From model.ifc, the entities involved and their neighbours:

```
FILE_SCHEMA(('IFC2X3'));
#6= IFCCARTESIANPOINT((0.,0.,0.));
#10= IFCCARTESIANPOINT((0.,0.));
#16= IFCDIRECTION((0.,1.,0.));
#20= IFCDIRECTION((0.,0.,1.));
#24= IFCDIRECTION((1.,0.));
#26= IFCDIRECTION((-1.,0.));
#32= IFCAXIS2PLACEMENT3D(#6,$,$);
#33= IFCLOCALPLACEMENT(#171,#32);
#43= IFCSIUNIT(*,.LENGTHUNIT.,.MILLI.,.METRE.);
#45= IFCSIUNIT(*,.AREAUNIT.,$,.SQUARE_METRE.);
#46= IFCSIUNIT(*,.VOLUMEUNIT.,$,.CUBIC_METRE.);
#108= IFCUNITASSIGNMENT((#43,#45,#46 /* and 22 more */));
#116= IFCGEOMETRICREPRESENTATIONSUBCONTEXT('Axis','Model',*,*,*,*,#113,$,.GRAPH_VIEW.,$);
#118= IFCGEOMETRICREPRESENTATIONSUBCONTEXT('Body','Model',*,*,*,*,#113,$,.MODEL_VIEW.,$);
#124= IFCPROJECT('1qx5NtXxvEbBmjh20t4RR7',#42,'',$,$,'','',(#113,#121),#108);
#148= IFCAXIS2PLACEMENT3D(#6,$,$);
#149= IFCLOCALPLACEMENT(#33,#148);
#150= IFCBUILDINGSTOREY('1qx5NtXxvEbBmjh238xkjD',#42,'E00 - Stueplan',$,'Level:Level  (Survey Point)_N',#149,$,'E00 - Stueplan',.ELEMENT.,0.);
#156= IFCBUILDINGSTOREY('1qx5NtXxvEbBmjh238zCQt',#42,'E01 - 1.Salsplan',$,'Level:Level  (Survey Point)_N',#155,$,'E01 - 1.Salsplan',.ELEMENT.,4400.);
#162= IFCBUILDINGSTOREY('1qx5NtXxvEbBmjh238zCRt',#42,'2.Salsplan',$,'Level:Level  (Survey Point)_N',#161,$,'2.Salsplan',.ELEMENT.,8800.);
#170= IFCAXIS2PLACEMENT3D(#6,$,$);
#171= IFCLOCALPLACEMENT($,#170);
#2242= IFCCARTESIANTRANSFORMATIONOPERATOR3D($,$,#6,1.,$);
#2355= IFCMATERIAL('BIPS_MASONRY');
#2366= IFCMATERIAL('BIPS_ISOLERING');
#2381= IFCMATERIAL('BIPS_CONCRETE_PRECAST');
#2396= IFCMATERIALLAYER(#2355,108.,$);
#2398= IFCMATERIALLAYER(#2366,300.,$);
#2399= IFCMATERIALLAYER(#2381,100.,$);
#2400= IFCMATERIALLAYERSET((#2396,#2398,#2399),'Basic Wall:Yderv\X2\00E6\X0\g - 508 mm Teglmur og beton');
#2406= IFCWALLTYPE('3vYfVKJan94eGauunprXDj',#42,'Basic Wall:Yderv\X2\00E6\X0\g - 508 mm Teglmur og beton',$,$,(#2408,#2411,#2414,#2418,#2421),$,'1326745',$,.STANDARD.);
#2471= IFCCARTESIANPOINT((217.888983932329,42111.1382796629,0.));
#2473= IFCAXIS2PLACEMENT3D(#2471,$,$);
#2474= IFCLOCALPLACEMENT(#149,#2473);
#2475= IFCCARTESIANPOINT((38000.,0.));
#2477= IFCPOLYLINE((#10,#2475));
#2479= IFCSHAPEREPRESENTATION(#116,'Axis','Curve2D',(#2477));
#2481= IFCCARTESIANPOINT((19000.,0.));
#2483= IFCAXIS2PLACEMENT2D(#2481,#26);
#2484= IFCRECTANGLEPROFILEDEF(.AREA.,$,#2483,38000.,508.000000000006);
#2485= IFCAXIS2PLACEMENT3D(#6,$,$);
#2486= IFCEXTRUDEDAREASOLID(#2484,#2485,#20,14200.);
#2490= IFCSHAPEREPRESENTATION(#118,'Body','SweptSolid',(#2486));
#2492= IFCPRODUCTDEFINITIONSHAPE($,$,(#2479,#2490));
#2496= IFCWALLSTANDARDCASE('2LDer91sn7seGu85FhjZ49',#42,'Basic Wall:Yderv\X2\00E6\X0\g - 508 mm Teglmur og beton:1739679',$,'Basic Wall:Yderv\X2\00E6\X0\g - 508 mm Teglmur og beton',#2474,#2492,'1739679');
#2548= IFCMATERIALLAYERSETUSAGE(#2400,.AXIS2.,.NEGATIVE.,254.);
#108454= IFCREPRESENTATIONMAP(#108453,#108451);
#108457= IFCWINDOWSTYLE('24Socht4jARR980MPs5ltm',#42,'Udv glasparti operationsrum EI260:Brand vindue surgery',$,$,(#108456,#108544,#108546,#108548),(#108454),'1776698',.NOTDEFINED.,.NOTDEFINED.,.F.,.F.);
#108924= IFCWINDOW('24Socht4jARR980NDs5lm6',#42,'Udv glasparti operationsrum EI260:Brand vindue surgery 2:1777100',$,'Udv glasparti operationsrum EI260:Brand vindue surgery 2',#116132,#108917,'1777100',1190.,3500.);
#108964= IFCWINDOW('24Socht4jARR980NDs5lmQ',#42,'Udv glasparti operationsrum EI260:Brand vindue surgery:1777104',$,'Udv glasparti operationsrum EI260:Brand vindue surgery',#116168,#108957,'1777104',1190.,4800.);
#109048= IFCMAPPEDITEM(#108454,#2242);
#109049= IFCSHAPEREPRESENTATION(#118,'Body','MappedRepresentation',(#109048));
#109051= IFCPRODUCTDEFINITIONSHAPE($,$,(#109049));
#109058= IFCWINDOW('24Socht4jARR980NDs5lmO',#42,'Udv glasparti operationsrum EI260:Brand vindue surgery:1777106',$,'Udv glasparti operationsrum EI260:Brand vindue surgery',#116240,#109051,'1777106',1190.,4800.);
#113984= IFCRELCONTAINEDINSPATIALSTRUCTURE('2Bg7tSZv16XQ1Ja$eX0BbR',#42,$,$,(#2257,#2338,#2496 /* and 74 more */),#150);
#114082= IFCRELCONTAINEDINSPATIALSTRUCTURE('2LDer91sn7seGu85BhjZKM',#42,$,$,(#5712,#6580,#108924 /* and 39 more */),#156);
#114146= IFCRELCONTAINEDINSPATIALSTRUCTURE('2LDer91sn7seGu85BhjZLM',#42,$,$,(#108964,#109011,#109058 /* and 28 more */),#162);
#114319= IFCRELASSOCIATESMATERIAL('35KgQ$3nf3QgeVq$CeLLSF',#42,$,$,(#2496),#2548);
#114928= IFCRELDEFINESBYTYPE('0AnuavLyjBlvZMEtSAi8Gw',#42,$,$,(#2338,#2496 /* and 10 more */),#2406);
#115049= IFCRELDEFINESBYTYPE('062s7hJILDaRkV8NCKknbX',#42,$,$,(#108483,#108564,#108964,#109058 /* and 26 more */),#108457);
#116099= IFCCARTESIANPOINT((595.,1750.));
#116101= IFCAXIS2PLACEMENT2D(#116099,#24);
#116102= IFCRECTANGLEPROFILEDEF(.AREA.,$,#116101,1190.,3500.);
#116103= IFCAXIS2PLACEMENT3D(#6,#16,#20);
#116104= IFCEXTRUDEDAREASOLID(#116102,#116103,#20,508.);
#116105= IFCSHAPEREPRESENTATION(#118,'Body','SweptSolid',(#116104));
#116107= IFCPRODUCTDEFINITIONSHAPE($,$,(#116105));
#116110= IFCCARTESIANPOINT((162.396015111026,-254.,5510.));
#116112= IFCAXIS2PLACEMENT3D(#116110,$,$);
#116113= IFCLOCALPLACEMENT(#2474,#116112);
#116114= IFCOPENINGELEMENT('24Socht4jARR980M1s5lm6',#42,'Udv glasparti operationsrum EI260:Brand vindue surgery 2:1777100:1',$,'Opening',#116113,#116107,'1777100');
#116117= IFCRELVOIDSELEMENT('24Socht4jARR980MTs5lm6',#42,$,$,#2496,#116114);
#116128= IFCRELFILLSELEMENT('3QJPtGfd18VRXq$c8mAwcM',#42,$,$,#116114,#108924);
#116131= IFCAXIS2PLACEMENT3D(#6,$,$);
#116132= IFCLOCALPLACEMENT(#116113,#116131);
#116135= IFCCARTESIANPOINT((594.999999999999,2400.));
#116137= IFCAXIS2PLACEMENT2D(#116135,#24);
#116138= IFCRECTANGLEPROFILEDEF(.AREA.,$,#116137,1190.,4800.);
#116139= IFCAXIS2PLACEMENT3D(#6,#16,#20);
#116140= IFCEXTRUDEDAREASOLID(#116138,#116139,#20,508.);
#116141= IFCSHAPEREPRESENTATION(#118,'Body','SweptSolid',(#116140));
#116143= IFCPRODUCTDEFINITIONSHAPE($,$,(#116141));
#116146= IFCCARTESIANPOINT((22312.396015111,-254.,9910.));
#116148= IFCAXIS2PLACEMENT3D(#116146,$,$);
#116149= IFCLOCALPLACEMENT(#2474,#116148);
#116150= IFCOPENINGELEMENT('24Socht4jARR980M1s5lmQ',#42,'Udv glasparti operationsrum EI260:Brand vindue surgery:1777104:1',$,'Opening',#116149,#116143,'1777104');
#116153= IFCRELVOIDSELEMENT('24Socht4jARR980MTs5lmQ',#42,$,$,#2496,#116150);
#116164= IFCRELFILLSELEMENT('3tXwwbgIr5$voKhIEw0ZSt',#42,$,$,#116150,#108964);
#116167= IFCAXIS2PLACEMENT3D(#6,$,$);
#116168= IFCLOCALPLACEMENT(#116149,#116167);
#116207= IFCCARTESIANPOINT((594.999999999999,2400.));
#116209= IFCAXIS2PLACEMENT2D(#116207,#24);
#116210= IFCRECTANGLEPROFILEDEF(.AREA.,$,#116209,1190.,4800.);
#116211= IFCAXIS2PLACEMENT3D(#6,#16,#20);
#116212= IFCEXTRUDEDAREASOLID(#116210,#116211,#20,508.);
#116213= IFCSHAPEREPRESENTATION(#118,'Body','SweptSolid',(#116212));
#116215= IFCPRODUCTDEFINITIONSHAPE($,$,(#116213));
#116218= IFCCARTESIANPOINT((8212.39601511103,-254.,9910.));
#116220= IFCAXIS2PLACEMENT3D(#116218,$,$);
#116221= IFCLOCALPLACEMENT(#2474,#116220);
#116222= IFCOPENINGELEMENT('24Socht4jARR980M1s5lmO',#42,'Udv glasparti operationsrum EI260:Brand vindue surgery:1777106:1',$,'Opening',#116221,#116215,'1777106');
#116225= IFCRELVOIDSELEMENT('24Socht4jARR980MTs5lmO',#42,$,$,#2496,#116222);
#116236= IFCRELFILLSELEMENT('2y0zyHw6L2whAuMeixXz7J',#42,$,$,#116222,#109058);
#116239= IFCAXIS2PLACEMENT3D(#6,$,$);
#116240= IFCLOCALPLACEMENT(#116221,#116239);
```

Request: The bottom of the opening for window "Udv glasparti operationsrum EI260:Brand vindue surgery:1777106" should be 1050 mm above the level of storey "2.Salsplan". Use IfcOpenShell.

```python
import numpy as np
import ifcopenshell
import ifcopenshell.api.geometry
import ifcopenshell.geom
import ifcopenshell.util.element
import ifcopenshell.util.placement
import ifcopenshell.util.shape
import ifcopenshell.util.unit

model = ifcopenshell.open("model.ifc")
unit_scale = ifcopenshell.util.unit.calculate_unit_scale(model)

window = model.by_guid("24Socht4jARR980NDs5lmO")
opening = window.FillsVoids[0].RelatingOpeningElement
storey = ifcopenshell.util.element.get_container(window, ifc_class="IfcBuildingStorey")
level = ifcopenshell.util.placement.get_local_placement(storey.ObjectPlacement)[2, 3]

# The opening's origin need not be at the sill, so measure its lowest point.
shape = ifcopenshell.geom.create_shape(ifcopenshell.geom.settings(), opening)
bottom = ifcopenshell.util.shape.get_shape_bottom_elevation(shape, shape.geometry) / unit_scale
dz = level + 1.05 / unit_scale - bottom

shift = np.array([0.0, 0.0, dz])
# The window is placed relative to its opening, so it follows when the opening moves.
matrix = ifcopenshell.util.placement.get_local_placement(opening.ObjectPlacement)
matrix[:3, 3] += shift
ifcopenshell.api.geometry.edit_object_placement(
    model, product=opening, matrix=matrix, is_si=False, should_transform_children=True
)

print(f"moved by {dz * unit_scale:+.3f} m")

model.write("model_rev.ifc")
```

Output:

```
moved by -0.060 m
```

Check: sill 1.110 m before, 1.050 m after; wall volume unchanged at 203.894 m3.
